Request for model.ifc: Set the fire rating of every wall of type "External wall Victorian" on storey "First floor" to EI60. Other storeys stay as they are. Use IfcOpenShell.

First a look at what the model holds.

```python
import ifcopenshell
import ifcopenshell.util.element

model = ifcopenshell.open("model.ifc")
print(model.schema)
storey = next(s for s in model.by_type("IfcBuildingStorey") if s.Name == "First floor")
walls = [e for e in ifcopenshell.util.element.get_decomposition(storey) if e.is_a("IfcWall")]
seen = {}
for e in walls:
    element_type = ifcopenshell.util.element.get_type(e)
    key = (element_type.Name if element_type != e and element_type else None, ifcopenshell.util.element.get_pset(e, "Pset_WallCommon", "FireRating"))
    seen[key] = seen.get(key, 0) + 1
for (name, value), count in sorted(seen.items(), key=str):
    print(count, "x", name, "|", value)
```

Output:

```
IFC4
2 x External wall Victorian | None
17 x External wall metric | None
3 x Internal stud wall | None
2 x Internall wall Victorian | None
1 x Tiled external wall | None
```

```python
import ifcopenshell
import ifcopenshell.api.pset
import ifcopenshell.util.element

model = ifcopenshell.open("model.ifc")

storey = next(s for s in model.by_type("IfcBuildingStorey") if s.Name == "First floor")
walls = [e for e in ifcopenshell.util.element.get_decomposition(storey) if e.is_a("IfcWall")]

count = 0
for e in walls:
    element_type = ifcopenshell.util.element.get_type(e)
    if element_type in (None, e) or element_type.Name != "External wall Victorian":
        continue
    # add_pset returns the element's existing set when there is one.
    pset = ifcopenshell.api.pset.add_pset(model, product=e, name="Pset_WallCommon")
    ifcopenshell.api.pset.edit_pset(model, pset=pset, properties={"FireRating": "EI60"})
    count += 1

print(count, "walls updated")

model.write("model-out.ifc")
```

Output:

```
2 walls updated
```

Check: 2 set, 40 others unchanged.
